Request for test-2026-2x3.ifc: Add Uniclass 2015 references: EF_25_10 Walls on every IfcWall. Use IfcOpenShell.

First a look at what the model holds.

```python
import ifcopenshell

model = ifcopenshell.open("test-2026-2x3.ifc")
print(model.schema)
print("classifications:", [c.Name for c in model.by_type("IfcClassification")])
for ifc_class in ("IfcDoor", "IfcRoof", "IfcStair", "IfcWall", "IfcWindow"):
    print(ifc_class, len(model.by_type(ifc_class)))
```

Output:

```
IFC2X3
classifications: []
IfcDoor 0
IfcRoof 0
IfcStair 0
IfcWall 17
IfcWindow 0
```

```python
import ifcopenshell
import ifcopenshell.api.classification

model = ifcopenshell.open("test-2026-2x3.ifc")

# IFC2X3 requires Source and Edition and has no link from the project to the system.
system = model.create_entity("IfcClassification", Source="NBS", Edition="2015", Name="Uniclass 2015")

codes = {
    "IfcWall": ("EF_25_10", "Walls"),
}
for ifc_class, (code, name) in codes.items():
    products = model.by_type(ifc_class)
    ifcopenshell.api.classification.add_reference(
        model, products=products, classification=system, identification=code, name=name
    )
    print(code, len(products))

model.write("test-2026-2x3_v2.ifc")
```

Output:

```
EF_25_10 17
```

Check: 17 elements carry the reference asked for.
